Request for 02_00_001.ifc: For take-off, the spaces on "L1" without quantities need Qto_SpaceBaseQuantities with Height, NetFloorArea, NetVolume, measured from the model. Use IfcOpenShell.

First a look at what the model holds.

```python
import ifcopenshell
import ifcopenshell.util.element
import ifcopenshell.util.unit

model = ifcopenshell.open("02_00_001.ifc")
print(model.schema)
for unit_type in ("LENGTHUNIT", "AREAUNIT", "VOLUMEUNIT"):
    print(unit_type, ifcopenshell.util.unit.calculate_unit_scale(model, unit_type))
storey = next(s for s in model.by_type("IfcBuildingStorey") if s.Name == "L1")
spaces = [e for e in ifcopenshell.util.element.get_decomposition(storey) if e.is_a("IfcSpace")]
for e in sorted(spaces, key=lambda e: e.id()):
    print(e.id(), e.is_a(), e.Name, list(ifcopenshell.util.element.get_psets(e, qtos_only=True)), sep=" | ")
```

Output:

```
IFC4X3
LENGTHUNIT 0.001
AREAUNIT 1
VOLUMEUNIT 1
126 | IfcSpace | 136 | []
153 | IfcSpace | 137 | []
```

```python
import ifcopenshell
import ifcopenshell.api.pset
import ifcopenshell.geom
import ifcopenshell.util.element
import ifcopenshell.util.shape
import ifcopenshell.util.unit

model = ifcopenshell.open("02_00_001.ifc")
unit_scale = ifcopenshell.util.unit.calculate_unit_scale(model)
area_scale = ifcopenshell.util.unit.calculate_unit_scale(model, "AREAUNIT")
volume_scale = ifcopenshell.util.unit.calculate_unit_scale(model, "VOLUMEUNIT")
settings = ifcopenshell.geom.settings()

storey = next(s for s in model.by_type("IfcBuildingStorey") if s.Name == "L1")
spaces = [e for e in ifcopenshell.util.element.get_decomposition(storey) if e.is_a("IfcSpace")]

for e in sorted(spaces, key=lambda e: e.id()):
    if ifcopenshell.util.element.get_psets(e, qtos_only=True, should_inherit=False):
        continue
    # Geometry comes back in metres, in the element's own axes.
    shape = ifcopenshell.geom.create_shape(settings, e)
    values = {
        "Height": ifcopenshell.util.shape.get_z(shape.geometry) / unit_scale,
        "NetFloorArea": ifcopenshell.util.shape.get_footprint_area(shape.geometry) / area_scale,
        "NetVolume": ifcopenshell.util.shape.get_volume(shape.geometry) / volume_scale,
    }
    qto = ifcopenshell.api.pset.add_qto(model, product=e, name="Qto_SpaceBaseQuantities")
    ifcopenshell.api.pset.edit_qto(model, qto=qto, properties=values)
    print(e.id(), {k: round(v, 3) for k, v in values.items()})

model.write("02_00_001_edited.ifc")
```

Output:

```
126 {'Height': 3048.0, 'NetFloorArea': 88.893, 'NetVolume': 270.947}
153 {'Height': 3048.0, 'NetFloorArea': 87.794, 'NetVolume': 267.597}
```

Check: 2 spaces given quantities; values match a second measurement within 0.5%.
